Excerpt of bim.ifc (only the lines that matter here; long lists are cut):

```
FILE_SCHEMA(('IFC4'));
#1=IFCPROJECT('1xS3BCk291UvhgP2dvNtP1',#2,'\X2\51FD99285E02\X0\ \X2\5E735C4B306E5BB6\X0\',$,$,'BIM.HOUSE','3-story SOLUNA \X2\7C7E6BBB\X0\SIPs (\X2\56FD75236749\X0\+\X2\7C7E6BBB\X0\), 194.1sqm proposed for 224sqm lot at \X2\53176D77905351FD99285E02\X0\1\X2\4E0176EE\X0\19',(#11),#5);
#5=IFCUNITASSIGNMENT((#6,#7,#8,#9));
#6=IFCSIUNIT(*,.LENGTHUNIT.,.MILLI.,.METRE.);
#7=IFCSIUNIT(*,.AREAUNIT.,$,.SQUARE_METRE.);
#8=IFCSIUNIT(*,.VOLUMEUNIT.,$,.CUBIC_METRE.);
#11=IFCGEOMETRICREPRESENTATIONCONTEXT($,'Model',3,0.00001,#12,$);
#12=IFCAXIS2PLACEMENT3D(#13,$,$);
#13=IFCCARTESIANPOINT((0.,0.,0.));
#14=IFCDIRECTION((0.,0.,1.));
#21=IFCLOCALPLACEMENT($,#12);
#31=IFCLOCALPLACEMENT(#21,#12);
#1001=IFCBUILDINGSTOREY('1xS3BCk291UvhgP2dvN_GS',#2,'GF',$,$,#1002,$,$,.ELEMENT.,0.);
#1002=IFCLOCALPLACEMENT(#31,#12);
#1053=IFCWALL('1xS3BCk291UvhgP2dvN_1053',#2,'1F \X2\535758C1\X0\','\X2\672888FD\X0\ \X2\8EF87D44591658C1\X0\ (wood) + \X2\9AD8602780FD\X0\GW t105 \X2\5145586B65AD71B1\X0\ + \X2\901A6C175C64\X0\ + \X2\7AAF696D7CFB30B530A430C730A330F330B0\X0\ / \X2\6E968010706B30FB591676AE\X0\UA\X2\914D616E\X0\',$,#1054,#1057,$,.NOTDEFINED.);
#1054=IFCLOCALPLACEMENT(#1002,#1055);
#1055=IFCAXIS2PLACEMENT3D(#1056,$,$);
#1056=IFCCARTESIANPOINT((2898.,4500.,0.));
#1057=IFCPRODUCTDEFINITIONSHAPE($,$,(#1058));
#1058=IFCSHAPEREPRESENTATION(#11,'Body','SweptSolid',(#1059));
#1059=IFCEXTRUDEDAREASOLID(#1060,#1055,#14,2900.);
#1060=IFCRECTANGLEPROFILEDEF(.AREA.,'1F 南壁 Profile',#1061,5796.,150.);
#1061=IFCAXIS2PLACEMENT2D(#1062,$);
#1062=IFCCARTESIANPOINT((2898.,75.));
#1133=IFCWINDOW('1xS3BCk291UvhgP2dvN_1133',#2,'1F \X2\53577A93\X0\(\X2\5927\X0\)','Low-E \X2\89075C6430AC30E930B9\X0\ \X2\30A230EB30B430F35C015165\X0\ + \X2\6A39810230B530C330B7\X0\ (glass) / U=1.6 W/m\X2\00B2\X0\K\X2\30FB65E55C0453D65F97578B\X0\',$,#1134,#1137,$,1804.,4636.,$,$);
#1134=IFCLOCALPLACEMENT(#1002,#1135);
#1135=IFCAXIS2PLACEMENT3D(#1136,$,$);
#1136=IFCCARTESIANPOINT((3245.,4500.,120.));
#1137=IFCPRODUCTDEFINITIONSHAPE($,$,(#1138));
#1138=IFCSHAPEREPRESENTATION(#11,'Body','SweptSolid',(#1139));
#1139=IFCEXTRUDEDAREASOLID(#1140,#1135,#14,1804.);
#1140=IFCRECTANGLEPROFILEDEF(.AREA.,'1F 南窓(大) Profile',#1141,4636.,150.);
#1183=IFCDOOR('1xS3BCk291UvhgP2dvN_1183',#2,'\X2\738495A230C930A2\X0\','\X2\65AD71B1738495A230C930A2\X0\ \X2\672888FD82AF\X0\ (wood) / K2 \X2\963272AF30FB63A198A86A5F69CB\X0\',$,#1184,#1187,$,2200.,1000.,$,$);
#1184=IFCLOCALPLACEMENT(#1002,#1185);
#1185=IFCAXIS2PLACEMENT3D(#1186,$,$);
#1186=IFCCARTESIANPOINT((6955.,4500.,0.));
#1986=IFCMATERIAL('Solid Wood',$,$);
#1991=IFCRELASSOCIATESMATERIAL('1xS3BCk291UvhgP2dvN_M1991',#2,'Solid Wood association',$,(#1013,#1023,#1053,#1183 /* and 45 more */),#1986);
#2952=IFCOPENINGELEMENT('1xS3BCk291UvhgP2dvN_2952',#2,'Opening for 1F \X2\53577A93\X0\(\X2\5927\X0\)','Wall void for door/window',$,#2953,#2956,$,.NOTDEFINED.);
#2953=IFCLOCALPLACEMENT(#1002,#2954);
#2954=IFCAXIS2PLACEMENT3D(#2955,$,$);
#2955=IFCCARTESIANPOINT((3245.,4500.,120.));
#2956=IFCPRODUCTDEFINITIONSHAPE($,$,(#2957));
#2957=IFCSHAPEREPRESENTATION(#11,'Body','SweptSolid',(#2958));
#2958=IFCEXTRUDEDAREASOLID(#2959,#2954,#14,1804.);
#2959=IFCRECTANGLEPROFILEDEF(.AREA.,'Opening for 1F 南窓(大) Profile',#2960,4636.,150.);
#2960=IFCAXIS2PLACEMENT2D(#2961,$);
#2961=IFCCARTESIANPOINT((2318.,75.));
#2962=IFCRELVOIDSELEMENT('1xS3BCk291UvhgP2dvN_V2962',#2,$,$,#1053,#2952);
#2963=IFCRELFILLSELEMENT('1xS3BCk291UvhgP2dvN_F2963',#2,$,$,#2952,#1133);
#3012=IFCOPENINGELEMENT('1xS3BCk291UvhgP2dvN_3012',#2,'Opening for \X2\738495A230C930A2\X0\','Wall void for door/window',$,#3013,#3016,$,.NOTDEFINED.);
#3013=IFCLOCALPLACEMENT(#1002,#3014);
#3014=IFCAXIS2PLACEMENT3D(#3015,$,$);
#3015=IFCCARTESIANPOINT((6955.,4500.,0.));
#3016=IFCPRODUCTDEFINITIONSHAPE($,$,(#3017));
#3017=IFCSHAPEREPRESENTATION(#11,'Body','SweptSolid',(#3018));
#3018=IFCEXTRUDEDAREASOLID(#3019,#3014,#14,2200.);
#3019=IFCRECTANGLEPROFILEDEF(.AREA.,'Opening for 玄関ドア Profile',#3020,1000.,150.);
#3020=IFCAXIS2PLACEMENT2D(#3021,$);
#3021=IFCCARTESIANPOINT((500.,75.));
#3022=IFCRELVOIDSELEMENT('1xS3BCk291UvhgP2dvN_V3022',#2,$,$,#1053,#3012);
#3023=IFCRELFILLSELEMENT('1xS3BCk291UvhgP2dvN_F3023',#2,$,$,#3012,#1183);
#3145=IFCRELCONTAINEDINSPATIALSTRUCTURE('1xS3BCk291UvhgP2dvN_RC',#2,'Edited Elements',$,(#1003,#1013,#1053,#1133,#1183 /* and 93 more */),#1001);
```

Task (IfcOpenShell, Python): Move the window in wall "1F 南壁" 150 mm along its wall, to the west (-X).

```python
import ifcopenshell
import ifcopenshell.api.geometry
import ifcopenshell.util.placement
import ifcopenshell.util.unit

model = ifcopenshell.open("bim.ifc")
unit_scale = ifcopenshell.util.unit.calculate_unit_scale(model)

window = model.by_guid("1xS3BCk291UvhgP2dvN_1133")
opening = window.FillsVoids[0].RelatingOpeningElement
wall = opening.VoidsElements[0].RelatingBuildingElement

wall_matrix = ifcopenshell.util.placement.get_local_placement(wall.ObjectPlacement)
shift = wall_matrix[:3, 0] * -0.15 / unit_scale
before = ifcopenshell.util.placement.get_local_placement(window.ObjectPlacement)[:3, 3].copy()

# The window is not placed relative to its opening, so move both.
for product in (opening, window):
    matrix = ifcopenshell.util.placement.get_local_placement(product.ObjectPlacement)
    matrix[:3, 3] += shift
    ifcopenshell.api.geometry.edit_object_placement(model, product=product, matrix=matrix, is_si=False)

after = ifcopenshell.util.placement.get_local_placement(window.ObjectPlacement)[:3, 3]
print("window moved by", (after - before).round(3) + 0.0)

model.write("bim_edited.ifc")
```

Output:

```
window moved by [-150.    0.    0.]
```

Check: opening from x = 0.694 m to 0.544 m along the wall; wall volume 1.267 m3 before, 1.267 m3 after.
